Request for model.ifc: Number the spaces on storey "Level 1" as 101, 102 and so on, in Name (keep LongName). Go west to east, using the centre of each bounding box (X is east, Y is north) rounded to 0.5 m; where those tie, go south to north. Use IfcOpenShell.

First a look at what the model holds.

```python
import ifcopenshell
import ifcopenshell.util.element
import ifcopenshell.util.placement

model = ifcopenshell.open("model.ifc")
print(model.schema)
storey = next(s for s in model.by_type("IfcBuildingStorey") if s.Name == "Level 1")
spaces = [e for e in ifcopenshell.util.element.get_decomposition(storey) if e.is_a("IfcSpace")]
for e in sorted(spaces, key=lambda e: e.id()):
    origin = ifcopenshell.util.placement.get_local_placement(e.ObjectPlacement)[:3, 3]
    print(e.id(), e.Name, e.LongName, origin.round(2) + 0.0, sep=" | ")
```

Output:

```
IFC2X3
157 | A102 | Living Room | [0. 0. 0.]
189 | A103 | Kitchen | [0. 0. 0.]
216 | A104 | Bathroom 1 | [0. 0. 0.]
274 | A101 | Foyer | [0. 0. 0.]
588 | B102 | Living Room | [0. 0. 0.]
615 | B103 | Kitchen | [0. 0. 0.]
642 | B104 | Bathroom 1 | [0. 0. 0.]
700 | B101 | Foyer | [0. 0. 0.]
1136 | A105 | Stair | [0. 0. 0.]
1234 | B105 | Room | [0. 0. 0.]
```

```python
import ifcopenshell
import ifcopenshell.geom
import ifcopenshell.util.element
import ifcopenshell.util.shape

model = ifcopenshell.open("model.ifc")
settings = ifcopenshell.geom.settings()
settings.set("use-world-coords", True)


def centre(element):
    shape = ifcopenshell.geom.create_shape(settings, element)
    return ifcopenshell.util.shape.get_bbox_centroid(shape.geometry)


storey = next(s for s in model.by_type("IfcBuildingStorey") if s.Name == "Level 1")
spaces = [e for e in ifcopenshell.util.element.get_decomposition(storey) if e.is_a("IfcSpace")]

# Insertion points can sit at a corner or the storey origin, so sort by the geometry (in metres).
centres = {e: centre(e) for e in spaces}
spaces.sort(key=lambda e: (round(centres[e][0] / 0.5), centres[e][1]))

for i, e in enumerate(spaces, start=1):
    number = f"1{i:02d}"
    e.Name = number
    print(e.id(), number)

model.write("model_updated.ifc")
```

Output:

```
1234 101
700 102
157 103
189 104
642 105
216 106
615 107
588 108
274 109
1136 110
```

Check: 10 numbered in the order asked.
